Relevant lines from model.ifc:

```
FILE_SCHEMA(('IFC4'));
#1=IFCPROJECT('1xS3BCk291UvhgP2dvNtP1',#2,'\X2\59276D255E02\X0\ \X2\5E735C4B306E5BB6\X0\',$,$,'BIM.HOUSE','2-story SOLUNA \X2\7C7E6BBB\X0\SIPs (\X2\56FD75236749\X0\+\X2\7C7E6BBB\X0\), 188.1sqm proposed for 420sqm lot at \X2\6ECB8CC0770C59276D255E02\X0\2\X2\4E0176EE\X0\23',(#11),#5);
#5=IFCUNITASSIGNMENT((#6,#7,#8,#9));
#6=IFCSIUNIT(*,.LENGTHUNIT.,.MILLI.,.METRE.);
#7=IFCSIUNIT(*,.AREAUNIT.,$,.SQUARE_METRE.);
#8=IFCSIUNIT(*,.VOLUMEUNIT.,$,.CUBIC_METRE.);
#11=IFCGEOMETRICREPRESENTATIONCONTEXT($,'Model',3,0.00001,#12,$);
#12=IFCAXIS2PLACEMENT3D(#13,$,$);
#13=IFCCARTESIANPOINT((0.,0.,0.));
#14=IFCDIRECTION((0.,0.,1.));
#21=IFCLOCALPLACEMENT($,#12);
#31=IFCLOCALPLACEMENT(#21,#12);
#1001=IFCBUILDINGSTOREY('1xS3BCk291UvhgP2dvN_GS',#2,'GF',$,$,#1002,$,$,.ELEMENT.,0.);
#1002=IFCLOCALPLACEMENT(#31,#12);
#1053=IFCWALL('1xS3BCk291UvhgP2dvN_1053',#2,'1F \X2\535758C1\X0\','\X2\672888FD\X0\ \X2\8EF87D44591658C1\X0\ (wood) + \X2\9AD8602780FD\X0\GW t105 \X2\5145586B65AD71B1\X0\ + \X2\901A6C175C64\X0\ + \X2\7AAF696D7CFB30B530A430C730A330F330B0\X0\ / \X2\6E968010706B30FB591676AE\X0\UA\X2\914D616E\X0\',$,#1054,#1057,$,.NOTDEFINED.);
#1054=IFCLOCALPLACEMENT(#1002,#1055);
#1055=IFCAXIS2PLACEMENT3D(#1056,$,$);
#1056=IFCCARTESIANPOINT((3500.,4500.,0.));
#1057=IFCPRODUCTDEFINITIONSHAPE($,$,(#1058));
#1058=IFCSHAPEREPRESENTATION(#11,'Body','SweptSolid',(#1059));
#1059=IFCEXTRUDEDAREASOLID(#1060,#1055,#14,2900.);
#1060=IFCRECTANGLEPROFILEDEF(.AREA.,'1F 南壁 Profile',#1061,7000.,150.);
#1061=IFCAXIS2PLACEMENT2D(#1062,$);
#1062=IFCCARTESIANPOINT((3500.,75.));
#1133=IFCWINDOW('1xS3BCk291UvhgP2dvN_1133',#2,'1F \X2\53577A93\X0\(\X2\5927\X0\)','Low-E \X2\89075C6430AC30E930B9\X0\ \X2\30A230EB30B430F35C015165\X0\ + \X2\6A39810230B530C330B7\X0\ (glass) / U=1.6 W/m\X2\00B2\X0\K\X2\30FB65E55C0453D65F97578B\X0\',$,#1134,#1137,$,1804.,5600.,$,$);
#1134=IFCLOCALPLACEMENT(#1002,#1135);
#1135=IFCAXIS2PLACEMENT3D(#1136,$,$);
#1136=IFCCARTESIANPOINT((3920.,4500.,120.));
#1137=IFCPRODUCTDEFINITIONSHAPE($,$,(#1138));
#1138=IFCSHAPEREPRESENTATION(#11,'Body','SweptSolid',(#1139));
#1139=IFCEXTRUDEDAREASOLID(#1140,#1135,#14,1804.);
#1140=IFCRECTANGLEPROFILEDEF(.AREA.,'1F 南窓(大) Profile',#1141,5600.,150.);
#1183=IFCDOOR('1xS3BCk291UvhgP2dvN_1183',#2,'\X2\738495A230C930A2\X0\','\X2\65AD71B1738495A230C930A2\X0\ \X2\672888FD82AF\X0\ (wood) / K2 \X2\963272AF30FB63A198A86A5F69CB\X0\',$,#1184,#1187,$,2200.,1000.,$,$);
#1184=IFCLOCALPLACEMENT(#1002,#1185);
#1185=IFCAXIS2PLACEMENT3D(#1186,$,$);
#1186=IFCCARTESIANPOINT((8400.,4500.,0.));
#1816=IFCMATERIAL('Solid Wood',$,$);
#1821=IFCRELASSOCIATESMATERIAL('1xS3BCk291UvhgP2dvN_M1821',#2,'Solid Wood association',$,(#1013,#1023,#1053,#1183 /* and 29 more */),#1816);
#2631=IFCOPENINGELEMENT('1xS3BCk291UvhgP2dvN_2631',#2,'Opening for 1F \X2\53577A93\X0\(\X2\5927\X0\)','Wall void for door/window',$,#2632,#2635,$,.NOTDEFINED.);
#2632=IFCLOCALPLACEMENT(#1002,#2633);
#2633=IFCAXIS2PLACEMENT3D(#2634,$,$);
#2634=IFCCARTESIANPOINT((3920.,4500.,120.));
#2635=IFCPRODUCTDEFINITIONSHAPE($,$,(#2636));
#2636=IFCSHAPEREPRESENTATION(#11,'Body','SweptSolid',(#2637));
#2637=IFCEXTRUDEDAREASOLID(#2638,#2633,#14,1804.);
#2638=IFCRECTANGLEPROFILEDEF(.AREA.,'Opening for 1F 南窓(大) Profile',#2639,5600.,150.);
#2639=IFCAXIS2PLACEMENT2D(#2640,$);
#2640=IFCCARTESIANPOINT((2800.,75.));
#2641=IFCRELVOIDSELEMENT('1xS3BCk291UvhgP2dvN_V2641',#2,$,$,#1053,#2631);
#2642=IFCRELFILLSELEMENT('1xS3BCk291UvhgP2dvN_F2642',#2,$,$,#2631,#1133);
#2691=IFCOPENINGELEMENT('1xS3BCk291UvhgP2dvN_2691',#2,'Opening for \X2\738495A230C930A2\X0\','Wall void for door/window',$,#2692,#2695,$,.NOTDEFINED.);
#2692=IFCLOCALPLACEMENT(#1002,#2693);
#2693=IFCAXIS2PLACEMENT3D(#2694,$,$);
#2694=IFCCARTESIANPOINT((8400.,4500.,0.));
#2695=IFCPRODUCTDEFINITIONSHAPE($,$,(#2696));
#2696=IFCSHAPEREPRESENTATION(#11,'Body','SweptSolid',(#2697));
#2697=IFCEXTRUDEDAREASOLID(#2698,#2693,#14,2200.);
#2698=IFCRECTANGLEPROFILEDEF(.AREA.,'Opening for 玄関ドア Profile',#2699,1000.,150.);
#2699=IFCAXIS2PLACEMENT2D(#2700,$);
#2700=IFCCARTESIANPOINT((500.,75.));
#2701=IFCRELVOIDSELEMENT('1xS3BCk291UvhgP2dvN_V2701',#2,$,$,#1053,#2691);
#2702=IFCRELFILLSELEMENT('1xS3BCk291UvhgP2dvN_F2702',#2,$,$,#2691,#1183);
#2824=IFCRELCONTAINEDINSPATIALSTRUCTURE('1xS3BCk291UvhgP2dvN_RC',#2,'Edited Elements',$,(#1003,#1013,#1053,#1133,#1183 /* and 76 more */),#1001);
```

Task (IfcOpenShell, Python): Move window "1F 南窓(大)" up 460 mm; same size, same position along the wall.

```python
import numpy as np
import ifcopenshell
import ifcopenshell.api.geometry
import ifcopenshell.util.placement
import ifcopenshell.util.unit

model = ifcopenshell.open("model.ifc")
unit_scale = ifcopenshell.util.unit.calculate_unit_scale(model)

window = model.by_guid("1xS3BCk291UvhgP2dvN_1133")
opening = window.FillsVoids[0].RelatingOpeningElement
dz = 0.46 / unit_scale

shift = np.array([0.0, 0.0, dz])
# The window is not placed relative to its opening, so move both.
for product in (opening, window):
    matrix = ifcopenshell.util.placement.get_local_placement(product.ObjectPlacement)
    matrix[:3, 3] += shift
    ifcopenshell.api.geometry.edit_object_placement(model, product=product, matrix=matrix, is_si=False)

print(f"moved by {dz * unit_scale:+.3f} m")

model.write("model_v2.ifc")
```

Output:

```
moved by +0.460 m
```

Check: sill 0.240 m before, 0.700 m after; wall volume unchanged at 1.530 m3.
